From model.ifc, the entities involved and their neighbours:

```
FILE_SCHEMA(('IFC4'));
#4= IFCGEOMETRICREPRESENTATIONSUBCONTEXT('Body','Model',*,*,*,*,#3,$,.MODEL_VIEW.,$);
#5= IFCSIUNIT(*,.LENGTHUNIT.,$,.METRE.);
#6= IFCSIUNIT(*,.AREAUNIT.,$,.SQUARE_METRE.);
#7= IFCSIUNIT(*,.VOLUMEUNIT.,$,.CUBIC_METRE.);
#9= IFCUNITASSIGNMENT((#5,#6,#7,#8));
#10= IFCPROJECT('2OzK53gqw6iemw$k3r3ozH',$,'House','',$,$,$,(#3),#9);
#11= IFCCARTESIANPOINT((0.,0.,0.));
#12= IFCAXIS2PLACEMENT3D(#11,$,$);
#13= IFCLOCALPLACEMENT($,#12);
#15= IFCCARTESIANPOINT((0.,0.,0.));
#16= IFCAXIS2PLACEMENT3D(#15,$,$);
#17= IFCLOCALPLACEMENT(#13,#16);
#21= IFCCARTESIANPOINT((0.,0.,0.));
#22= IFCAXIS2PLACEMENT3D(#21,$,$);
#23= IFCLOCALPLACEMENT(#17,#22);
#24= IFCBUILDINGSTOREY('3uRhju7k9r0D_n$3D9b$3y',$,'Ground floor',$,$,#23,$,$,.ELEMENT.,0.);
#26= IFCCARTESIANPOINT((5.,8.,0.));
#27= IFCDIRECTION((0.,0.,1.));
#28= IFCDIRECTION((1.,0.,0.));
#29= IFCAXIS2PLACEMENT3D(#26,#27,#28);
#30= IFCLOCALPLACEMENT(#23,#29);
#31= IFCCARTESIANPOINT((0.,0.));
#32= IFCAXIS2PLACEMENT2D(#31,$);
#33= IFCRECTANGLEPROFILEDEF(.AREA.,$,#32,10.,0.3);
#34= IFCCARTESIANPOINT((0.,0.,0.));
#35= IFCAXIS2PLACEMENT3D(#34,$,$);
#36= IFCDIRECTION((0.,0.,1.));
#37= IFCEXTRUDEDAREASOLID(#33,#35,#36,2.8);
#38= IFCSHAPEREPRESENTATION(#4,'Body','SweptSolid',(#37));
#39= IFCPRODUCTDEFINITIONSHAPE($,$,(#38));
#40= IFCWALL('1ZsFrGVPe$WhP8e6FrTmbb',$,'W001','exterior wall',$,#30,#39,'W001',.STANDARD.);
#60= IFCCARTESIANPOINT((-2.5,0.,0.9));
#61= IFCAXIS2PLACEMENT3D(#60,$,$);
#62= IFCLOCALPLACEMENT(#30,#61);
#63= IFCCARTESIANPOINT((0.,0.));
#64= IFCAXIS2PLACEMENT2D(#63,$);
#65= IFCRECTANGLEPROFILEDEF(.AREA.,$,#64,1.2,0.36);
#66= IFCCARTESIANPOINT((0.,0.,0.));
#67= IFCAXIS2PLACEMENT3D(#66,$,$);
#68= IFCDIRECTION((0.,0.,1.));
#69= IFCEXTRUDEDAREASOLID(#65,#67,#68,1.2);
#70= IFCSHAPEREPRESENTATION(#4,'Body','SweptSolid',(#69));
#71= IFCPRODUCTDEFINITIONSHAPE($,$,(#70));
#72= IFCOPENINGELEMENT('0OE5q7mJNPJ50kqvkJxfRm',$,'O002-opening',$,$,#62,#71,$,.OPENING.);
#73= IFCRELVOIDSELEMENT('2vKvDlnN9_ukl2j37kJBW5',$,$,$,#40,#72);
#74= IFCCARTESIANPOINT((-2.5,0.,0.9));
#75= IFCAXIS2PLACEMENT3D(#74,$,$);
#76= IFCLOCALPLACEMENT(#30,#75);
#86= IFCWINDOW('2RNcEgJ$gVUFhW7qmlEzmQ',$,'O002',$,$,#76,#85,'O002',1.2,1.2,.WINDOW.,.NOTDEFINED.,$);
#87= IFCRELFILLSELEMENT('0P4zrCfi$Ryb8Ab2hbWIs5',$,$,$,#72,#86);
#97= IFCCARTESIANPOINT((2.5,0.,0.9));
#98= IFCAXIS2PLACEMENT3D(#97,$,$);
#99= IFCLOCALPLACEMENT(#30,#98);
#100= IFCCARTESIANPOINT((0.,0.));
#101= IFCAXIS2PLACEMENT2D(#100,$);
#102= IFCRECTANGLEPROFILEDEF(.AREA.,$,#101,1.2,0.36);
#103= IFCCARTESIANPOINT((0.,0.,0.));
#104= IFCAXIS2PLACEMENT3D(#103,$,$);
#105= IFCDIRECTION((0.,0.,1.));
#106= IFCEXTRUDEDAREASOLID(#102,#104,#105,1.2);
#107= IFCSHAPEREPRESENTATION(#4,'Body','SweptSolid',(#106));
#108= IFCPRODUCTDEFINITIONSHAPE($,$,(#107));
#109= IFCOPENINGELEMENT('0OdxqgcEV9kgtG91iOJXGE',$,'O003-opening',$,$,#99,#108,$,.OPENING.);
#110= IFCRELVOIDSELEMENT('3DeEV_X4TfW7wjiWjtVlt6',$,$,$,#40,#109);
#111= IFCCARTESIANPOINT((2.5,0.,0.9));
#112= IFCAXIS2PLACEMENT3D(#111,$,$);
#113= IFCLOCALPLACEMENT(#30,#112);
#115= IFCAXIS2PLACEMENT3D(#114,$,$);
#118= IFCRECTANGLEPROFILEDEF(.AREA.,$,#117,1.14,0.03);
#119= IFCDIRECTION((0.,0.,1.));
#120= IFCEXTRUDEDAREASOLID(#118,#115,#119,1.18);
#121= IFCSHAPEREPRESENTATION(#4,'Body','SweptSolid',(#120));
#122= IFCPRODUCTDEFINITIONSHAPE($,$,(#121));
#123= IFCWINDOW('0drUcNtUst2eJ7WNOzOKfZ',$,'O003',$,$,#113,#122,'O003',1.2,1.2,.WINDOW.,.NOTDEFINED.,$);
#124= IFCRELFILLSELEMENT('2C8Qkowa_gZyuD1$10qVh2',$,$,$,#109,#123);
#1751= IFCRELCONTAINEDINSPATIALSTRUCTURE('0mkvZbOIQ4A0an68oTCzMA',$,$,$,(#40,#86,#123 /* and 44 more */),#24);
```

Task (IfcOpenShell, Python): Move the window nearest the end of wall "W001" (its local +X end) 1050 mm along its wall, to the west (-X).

```python
import ifcopenshell
import ifcopenshell.api.geometry
import ifcopenshell.util.placement

model = ifcopenshell.open("model.ifc")

window = model.by_id(123)
opening = window.FillsVoids[0].RelatingOpeningElement
wall = opening.VoidsElements[0].RelatingBuildingElement

wall_matrix = ifcopenshell.util.placement.get_local_placement(wall.ObjectPlacement)
shift = wall_matrix[:3, 0] * -1.05
before = ifcopenshell.util.placement.get_local_placement(window.ObjectPlacement)[:3, 3].copy()

# The window is not placed relative to its opening, so move both.
for product in (opening, window):
    matrix = ifcopenshell.util.placement.get_local_placement(product.ObjectPlacement)
    matrix[:3, 3] += shift
    ifcopenshell.api.geometry.edit_object_placement(model, product=product, matrix=matrix, is_si=False)

after = ifcopenshell.util.placement.get_local_placement(window.ObjectPlacement)[:3, 3]
print("window moved by", (after - before).round(3) + 0.0)

model.write("model_edited.ifc")
```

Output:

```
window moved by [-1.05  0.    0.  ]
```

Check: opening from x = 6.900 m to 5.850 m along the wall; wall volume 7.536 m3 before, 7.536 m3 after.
